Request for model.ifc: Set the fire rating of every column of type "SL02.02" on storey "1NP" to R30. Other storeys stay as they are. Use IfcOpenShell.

First a look at what the model holds.

```python
import ifcopenshell
import ifcopenshell.util.element

model = ifcopenshell.open("model.ifc")
print(model.schema)
storey = next(s for s in model.by_type("IfcBuildingStorey") if s.Name == "1NP")
columns = [e for e in ifcopenshell.util.element.get_decomposition(storey) if e.is_a("IfcColumn")]
seen = {}
for e in columns:
    element_type = ifcopenshell.util.element.get_type(e)
    key = (element_type.Name if element_type != e and element_type else None, ifcopenshell.util.element.get_pset(e, "Pset_ColumnCommon", "FireRating"))
    seen[key] = seen.get(key, 0) + 1
for (name, value), count in sorted(seen.items(), key=str):
    print(count, "x", name, "|", value)
```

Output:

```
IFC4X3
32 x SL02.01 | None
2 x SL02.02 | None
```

```python
import ifcopenshell
import ifcopenshell.api.pset
import ifcopenshell.util.element

model = ifcopenshell.open("model.ifc")

storey = next(s for s in model.by_type("IfcBuildingStorey") if s.Name == "1NP")
columns = [e for e in ifcopenshell.util.element.get_decomposition(storey) if e.is_a("IfcColumn")]

count = 0
for e in columns:
    element_type = ifcopenshell.util.element.get_type(e)
    if element_type in (None, e) or element_type.Name != "SL02.02":
        continue
    # add_pset returns the element's existing set when there is one.
    pset = ifcopenshell.api.pset.add_pset(model, product=e, name="Pset_ColumnCommon")
    ifcopenshell.api.pset.edit_pset(model, pset=pset, properties={"FireRating": "R30"})
    count += 1

print(count, "columns updated")

model.write("model_v2.ifc")
```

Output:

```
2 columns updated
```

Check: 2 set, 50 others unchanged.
